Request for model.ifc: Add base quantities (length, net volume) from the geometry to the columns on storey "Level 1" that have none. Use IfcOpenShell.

First a look at what the model holds.

```python
import ifcopenshell
import ifcopenshell.util.element
import ifcopenshell.util.unit

model = ifcopenshell.open("model.ifc")
print(model.schema)
for unit_type in ("LENGTHUNIT", "AREAUNIT", "VOLUMEUNIT"):
    print(unit_type, ifcopenshell.util.unit.calculate_unit_scale(model, unit_type))
storey = next(s for s in model.by_type("IfcBuildingStorey") if s.Name == "Level 1")
columns = [e for e in ifcopenshell.util.element.get_decomposition(storey) if e.is_a("IfcColumn")]
for e in sorted(columns, key=lambda e: e.id()):
    print(e.id(), e.is_a(), e.Name, list(ifcopenshell.util.element.get_psets(e, qtos_only=True)), sep=" | ")
```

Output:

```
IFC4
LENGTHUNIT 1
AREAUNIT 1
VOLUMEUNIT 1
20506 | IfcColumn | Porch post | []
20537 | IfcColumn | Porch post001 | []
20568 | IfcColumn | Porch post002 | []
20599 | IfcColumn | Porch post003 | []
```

```python
import ifcopenshell
import ifcopenshell.api.pset
import ifcopenshell.geom
import ifcopenshell.util.element
import ifcopenshell.util.shape
import ifcopenshell.util.unit

model = ifcopenshell.open("model.ifc")
unit_scale = ifcopenshell.util.unit.calculate_unit_scale(model)
volume_scale = ifcopenshell.util.unit.calculate_unit_scale(model, "VOLUMEUNIT")
settings = ifcopenshell.geom.settings()

storey = next(s for s in model.by_type("IfcBuildingStorey") if s.Name == "Level 1")
columns = [e for e in ifcopenshell.util.element.get_decomposition(storey) if e.is_a("IfcColumn")]

for e in sorted(columns, key=lambda e: e.id()):
    if ifcopenshell.util.element.get_psets(e, qtos_only=True, should_inherit=False):
        continue
    # Geometry comes back in metres, in the element's own axes.
    shape = ifcopenshell.geom.create_shape(settings, e)
    values = {
        "Length": ifcopenshell.util.shape.get_z(shape.geometry) / unit_scale,
        "NetVolume": ifcopenshell.util.shape.get_volume(shape.geometry) / volume_scale,
    }
    qto = ifcopenshell.api.pset.add_qto(model, product=e, name="Qto_ColumnBaseQuantities")
    ifcopenshell.api.pset.edit_qto(model, qto=qto, properties=values)
    print(e.id(), {k: round(v, 3) for k, v in values.items()})

model.write("model_v2.ifc")
```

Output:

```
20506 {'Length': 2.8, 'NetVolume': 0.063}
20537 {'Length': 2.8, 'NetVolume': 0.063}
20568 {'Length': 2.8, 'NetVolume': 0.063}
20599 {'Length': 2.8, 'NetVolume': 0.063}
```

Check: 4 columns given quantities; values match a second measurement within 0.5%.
